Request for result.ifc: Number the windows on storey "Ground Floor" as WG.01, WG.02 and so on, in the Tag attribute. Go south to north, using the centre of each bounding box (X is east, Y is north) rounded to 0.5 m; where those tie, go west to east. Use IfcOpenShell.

First a look at what the model holds.

```python
import ifcopenshell
import ifcopenshell.util.element
import ifcopenshell.util.placement

model = ifcopenshell.open("result.ifc")
print(model.schema)
storey = next(s for s in model.by_type("IfcBuildingStorey") if s.Name == "Ground Floor")
windows = [e for e in ifcopenshell.util.element.get_decomposition(storey) if e.is_a("IfcWindow")]
for e in sorted(windows, key=lambda e: e.id()):
    origin = ifcopenshell.util.placement.get_local_placement(e.ObjectPlacement)[:3, 3]
    print(e.id(), e.Tag, e.Name, origin.round(2) + 0.0, sep=" | ")
```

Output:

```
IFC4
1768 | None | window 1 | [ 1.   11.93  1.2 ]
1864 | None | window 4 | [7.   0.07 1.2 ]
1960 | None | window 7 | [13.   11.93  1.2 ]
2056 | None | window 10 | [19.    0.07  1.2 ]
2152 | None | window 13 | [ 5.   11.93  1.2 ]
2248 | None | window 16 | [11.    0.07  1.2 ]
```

```python
import ifcopenshell
import ifcopenshell.geom
import ifcopenshell.util.element
import ifcopenshell.util.shape

model = ifcopenshell.open("result.ifc")
settings = ifcopenshell.geom.settings()
settings.set("use-world-coords", True)


def centre(element):
    shape = ifcopenshell.geom.create_shape(settings, element)
    return ifcopenshell.util.shape.get_bbox_centroid(shape.geometry)


storey = next(s for s in model.by_type("IfcBuildingStorey") if s.Name == "Ground Floor")
windows = [e for e in ifcopenshell.util.element.get_decomposition(storey) if e.is_a("IfcWindow")]

# Insertion points can sit at a corner or the storey origin, so sort by the geometry (in metres).
centres = {e: centre(e) for e in windows}
windows.sort(key=lambda e: (round(centres[e][1] / 0.5), centres[e][0]))

for i, e in enumerate(windows, start=1):
    number = f"WG.{i:02d}"
    e.Tag = number
    print(e.id(), number)

model.write("result_updated.ifc")
```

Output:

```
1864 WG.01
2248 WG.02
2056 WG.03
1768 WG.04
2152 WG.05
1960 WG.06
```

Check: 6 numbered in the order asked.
